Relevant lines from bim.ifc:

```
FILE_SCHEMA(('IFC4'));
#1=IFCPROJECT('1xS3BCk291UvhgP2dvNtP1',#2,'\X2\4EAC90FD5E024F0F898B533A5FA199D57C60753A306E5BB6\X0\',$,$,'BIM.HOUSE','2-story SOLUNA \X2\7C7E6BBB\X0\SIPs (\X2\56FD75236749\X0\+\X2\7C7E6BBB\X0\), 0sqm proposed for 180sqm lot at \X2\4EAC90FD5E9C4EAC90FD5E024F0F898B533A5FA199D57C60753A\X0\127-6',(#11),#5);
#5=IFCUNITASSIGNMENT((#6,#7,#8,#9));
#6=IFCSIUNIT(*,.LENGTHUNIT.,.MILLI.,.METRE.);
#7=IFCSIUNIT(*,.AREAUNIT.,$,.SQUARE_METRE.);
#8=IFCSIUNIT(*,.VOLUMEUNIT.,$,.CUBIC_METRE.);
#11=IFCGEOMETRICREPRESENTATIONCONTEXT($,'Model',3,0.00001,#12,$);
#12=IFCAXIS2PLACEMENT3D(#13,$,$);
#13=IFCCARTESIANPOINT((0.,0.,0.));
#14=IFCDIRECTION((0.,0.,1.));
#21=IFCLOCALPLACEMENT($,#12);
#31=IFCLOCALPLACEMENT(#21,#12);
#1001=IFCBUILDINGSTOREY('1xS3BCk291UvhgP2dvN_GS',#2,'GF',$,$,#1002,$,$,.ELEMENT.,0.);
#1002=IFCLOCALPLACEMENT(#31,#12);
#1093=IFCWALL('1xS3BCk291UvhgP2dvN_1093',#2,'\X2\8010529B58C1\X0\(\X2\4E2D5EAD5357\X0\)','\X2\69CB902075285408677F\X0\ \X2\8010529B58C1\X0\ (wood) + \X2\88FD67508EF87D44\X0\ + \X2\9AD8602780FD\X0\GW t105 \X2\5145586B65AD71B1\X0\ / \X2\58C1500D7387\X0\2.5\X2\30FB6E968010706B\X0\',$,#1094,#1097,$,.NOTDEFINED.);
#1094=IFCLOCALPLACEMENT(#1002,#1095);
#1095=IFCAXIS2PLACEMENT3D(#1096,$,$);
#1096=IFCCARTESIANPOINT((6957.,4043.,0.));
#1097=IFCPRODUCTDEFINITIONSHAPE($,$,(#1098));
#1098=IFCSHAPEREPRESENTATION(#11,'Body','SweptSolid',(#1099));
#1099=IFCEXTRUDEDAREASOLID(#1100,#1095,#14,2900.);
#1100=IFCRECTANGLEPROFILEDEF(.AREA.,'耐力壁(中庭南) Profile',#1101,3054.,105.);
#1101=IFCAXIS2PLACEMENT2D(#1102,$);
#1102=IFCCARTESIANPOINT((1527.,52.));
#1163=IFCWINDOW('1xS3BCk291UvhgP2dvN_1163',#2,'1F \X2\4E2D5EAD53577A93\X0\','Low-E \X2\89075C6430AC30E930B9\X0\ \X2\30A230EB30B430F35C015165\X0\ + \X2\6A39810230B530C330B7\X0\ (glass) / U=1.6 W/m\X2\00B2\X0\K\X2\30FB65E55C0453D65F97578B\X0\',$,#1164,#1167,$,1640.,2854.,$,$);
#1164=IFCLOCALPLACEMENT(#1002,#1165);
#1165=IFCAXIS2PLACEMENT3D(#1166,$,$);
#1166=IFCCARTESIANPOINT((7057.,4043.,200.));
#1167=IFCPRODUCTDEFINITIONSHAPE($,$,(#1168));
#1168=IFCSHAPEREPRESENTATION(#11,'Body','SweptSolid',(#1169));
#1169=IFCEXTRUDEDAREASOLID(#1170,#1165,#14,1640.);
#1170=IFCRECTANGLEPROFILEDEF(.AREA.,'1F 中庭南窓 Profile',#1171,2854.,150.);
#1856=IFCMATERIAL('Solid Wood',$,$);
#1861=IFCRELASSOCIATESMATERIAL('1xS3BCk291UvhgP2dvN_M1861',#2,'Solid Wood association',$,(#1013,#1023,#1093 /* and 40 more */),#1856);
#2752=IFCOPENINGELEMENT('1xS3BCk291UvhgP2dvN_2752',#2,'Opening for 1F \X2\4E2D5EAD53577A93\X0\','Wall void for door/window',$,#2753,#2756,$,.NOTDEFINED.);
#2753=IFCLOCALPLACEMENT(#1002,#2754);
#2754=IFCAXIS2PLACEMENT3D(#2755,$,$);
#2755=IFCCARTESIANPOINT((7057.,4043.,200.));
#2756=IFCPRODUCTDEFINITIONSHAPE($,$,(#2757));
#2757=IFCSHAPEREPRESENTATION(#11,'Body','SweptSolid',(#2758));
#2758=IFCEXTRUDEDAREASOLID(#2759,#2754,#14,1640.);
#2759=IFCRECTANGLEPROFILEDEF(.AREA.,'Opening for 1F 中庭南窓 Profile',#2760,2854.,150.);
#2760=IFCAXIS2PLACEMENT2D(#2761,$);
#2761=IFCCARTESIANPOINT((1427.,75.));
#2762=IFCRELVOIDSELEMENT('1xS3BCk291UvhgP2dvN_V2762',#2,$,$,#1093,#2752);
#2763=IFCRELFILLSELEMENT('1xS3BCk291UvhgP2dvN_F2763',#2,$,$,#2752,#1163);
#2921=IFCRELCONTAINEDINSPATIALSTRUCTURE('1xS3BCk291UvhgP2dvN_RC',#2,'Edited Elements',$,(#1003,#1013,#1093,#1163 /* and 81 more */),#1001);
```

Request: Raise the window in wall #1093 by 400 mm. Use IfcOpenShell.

```python
import numpy as np
import ifcopenshell
import ifcopenshell.api.geometry
import ifcopenshell.util.placement
import ifcopenshell.util.unit

model = ifcopenshell.open("bim.ifc")
unit_scale = ifcopenshell.util.unit.calculate_unit_scale(model)

window = model.by_guid("1xS3BCk291UvhgP2dvN_1163")
opening = window.FillsVoids[0].RelatingOpeningElement
dz = 400.0

shift = np.array([0.0, 0.0, dz])
# The window is not placed relative to its opening, so move both.
for product in (opening, window):
    matrix = ifcopenshell.util.placement.get_local_placement(product.ObjectPlacement)
    matrix[:3, 3] += shift
    ifcopenshell.api.geometry.edit_object_placement(model, product=product, matrix=matrix, is_si=False)

print(f"moved by {dz * unit_scale:+.3f} m")

model.write("bim_v2.ifc")
```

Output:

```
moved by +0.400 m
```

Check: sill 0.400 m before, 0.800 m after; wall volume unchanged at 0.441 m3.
